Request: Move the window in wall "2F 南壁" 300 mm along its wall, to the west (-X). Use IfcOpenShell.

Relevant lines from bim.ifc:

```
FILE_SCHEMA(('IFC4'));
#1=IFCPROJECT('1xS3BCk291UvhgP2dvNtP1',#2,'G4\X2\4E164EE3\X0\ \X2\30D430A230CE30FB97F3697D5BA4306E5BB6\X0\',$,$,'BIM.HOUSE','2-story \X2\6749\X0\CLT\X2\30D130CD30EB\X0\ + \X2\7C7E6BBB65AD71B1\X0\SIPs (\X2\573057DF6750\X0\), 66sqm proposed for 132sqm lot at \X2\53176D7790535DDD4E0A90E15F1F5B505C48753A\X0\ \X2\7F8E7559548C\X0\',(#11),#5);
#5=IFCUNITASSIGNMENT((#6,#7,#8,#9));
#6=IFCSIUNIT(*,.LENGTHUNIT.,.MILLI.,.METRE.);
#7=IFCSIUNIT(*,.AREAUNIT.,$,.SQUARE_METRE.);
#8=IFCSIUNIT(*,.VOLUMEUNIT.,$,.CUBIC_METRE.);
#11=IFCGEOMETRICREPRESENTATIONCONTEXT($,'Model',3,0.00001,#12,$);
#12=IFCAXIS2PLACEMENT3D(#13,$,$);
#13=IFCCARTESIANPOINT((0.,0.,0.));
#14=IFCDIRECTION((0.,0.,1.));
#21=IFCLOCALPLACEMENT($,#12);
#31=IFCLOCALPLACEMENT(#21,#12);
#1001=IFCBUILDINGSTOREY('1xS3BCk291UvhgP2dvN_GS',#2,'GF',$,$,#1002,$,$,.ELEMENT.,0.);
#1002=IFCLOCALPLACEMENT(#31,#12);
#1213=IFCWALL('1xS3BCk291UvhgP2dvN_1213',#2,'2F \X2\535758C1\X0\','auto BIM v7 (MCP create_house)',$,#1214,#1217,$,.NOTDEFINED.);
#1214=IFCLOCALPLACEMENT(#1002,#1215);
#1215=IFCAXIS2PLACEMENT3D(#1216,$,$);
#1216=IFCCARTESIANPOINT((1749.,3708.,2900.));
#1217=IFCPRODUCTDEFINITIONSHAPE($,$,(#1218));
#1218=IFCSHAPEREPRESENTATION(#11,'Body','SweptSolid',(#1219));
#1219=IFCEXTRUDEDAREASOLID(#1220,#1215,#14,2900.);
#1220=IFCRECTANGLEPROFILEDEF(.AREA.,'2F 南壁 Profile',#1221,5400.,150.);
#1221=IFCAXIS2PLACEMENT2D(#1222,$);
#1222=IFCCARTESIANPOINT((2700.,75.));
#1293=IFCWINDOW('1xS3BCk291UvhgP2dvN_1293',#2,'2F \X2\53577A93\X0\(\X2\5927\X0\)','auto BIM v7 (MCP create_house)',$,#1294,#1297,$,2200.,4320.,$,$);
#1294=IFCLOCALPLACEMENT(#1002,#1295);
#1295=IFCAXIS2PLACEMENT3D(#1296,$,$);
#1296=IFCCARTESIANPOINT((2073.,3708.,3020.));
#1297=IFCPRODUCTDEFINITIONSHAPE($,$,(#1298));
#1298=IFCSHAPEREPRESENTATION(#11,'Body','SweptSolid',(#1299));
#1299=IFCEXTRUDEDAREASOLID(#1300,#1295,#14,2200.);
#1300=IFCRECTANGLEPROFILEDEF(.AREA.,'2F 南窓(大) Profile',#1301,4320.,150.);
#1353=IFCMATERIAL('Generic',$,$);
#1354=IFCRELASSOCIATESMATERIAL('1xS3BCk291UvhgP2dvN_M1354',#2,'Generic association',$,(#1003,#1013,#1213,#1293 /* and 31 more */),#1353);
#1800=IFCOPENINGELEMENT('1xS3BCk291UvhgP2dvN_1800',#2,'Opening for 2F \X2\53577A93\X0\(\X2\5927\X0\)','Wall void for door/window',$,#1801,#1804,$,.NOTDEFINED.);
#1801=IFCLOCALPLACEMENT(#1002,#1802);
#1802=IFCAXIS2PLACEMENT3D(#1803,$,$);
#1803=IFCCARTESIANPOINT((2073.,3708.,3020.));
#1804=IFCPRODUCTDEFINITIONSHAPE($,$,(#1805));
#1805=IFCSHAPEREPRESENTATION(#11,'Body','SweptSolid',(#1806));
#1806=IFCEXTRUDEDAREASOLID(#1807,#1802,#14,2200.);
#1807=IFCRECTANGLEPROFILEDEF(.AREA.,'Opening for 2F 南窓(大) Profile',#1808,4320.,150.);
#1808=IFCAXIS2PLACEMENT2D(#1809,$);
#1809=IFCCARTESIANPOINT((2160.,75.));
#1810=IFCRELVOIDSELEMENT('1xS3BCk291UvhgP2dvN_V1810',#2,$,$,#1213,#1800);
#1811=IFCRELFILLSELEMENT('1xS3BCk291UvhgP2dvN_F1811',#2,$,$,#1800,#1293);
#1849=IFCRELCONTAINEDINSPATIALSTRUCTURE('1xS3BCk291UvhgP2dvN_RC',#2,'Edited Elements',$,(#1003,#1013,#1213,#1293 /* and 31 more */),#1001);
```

```python
import ifcopenshell
import ifcopenshell.api.geometry
import ifcopenshell.util.placement

model = ifcopenshell.open("bim.ifc")

window = model.by_guid("1xS3BCk291UvhgP2dvN_1293")
opening = window.FillsVoids[0].RelatingOpeningElement
wall = opening.VoidsElements[0].RelatingBuildingElement

wall_matrix = ifcopenshell.util.placement.get_local_placement(wall.ObjectPlacement)
shift = wall_matrix[:3, 0] * -300.0
before = ifcopenshell.util.placement.get_local_placement(window.ObjectPlacement)[:3, 3].copy()

# The window is not placed relative to its opening, so move both.
for product in (opening, window):
    matrix = ifcopenshell.util.placement.get_local_placement(product.ObjectPlacement)
    matrix[:3, 3] += shift
    ifcopenshell.api.geometry.edit_object_placement(model, product=product, matrix=matrix, is_si=False)

after = ifcopenshell.util.placement.get_local_placement(window.ObjectPlacement)[:3, 3]
print("window moved by", (after - before).round(3) + 0.0)

model.write("bim_rev.ifc")
```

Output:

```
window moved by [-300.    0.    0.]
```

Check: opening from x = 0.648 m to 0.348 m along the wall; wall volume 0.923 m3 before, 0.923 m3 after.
